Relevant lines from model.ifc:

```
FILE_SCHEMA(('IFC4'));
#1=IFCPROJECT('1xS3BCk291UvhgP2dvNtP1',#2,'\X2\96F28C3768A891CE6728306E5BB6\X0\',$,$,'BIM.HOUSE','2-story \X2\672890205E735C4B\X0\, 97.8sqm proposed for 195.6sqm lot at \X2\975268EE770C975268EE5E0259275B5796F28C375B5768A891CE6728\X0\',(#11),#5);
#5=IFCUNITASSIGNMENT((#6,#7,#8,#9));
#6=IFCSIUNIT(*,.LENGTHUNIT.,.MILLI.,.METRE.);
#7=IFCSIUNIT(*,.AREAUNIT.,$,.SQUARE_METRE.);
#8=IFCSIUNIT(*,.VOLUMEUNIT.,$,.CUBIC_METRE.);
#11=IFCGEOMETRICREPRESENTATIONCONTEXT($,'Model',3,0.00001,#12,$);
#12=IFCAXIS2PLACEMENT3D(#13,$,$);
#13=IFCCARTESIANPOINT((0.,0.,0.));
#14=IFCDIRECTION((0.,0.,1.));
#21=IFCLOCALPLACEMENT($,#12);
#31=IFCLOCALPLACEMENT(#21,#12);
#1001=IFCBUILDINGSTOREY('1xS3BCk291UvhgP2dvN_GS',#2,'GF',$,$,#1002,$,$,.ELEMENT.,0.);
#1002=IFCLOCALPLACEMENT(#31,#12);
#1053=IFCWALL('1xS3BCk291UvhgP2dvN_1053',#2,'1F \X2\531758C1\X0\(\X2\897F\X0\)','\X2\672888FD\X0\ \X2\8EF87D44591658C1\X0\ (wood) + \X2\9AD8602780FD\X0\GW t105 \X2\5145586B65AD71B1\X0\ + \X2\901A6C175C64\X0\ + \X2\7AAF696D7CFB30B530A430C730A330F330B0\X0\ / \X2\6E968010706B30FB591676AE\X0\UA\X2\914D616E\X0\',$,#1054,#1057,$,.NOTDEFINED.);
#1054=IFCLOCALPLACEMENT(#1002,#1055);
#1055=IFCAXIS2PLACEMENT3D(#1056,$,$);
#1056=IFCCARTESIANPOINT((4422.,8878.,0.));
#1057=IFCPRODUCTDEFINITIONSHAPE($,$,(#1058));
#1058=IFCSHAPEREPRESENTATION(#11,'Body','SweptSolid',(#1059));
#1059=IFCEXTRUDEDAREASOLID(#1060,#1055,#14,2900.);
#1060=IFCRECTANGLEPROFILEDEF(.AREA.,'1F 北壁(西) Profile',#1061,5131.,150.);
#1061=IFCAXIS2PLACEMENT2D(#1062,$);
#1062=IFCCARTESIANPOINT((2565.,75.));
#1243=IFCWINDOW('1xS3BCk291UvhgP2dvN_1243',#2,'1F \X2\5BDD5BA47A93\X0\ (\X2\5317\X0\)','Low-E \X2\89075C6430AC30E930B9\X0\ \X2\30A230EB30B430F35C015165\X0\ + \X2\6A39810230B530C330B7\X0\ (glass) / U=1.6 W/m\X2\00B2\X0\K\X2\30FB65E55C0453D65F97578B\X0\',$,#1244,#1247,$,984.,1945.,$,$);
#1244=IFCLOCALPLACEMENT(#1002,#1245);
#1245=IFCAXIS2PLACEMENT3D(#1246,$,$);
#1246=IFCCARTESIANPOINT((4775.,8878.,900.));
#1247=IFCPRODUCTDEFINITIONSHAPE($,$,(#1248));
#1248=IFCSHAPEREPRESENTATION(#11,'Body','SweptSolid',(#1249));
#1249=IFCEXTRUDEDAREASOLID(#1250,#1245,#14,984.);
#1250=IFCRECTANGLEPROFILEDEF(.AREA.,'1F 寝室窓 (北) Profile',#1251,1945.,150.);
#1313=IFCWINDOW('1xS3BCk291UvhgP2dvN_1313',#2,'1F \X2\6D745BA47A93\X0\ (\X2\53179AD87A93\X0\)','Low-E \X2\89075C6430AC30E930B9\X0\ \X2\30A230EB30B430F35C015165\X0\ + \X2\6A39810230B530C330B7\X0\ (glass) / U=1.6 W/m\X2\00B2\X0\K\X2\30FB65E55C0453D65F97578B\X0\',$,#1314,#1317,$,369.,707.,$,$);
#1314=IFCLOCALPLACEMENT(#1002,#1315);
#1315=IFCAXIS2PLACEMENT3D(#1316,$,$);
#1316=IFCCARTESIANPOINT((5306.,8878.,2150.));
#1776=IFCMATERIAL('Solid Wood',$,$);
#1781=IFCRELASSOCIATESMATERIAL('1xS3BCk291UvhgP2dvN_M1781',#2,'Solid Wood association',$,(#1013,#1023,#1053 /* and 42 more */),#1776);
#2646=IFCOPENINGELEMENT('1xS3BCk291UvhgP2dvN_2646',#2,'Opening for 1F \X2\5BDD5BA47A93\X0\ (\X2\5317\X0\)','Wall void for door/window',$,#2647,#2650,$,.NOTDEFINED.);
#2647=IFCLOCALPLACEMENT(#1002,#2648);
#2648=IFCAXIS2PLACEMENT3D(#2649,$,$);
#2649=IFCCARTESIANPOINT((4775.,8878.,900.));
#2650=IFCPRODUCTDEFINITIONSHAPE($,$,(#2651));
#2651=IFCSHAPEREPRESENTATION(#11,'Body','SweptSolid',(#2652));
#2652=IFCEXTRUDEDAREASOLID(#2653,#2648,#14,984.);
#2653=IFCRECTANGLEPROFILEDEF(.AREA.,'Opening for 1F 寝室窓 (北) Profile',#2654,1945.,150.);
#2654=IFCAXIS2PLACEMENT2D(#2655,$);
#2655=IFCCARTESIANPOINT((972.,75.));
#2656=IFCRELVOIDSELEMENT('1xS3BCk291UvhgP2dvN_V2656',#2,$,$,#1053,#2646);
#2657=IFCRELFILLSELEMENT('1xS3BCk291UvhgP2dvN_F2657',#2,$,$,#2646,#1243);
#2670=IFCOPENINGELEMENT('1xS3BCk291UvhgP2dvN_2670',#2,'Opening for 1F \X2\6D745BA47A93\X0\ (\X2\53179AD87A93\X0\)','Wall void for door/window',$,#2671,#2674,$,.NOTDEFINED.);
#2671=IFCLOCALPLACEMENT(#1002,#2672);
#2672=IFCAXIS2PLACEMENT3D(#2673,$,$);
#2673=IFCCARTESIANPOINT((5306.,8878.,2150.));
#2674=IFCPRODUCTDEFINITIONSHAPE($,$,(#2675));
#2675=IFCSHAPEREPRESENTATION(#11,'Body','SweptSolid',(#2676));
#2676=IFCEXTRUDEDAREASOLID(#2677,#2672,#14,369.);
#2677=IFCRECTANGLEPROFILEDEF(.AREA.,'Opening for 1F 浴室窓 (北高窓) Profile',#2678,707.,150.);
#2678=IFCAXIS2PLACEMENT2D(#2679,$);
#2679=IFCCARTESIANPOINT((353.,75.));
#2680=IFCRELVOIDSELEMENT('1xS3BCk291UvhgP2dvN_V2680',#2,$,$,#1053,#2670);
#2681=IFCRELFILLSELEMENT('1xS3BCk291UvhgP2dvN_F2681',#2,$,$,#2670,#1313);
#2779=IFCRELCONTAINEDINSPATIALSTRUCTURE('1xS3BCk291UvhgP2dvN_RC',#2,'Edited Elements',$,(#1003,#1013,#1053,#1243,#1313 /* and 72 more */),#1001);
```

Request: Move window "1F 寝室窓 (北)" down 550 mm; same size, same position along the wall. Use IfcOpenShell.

```python
import numpy as np
import ifcopenshell
import ifcopenshell.api.geometry
import ifcopenshell.util.placement
import ifcopenshell.util.unit

model = ifcopenshell.open("model.ifc")
unit_scale = ifcopenshell.util.unit.calculate_unit_scale(model)

window = model.by_guid("1xS3BCk291UvhgP2dvN_1243")
opening = window.FillsVoids[0].RelatingOpeningElement
dz = -550.0

shift = np.array([0.0, 0.0, dz])
# The window is not placed relative to its opening, so move both.
for product in (opening, window):
    matrix = ifcopenshell.util.placement.get_local_placement(product.ObjectPlacement)
    matrix[:3, 3] += shift
    ifcopenshell.api.geometry.edit_object_placement(model, product=product, matrix=matrix, is_si=False)

print(f"moved by {dz * unit_scale:+.3f} m")

model.write("model_updated.ifc")
```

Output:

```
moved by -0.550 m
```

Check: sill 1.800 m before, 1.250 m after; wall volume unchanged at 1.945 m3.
